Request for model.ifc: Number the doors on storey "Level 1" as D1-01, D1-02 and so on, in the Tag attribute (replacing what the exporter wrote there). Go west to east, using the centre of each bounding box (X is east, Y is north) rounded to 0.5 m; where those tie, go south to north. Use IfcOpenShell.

First a look at what the model holds.

```python
import ifcopenshell
import ifcopenshell.util.element
import ifcopenshell.util.placement

model = ifcopenshell.open("model.ifc")
print(model.schema)
storey = next(s for s in model.by_type("IfcBuildingStorey") if s.Name == "Level 1")
doors = [e for e in ifcopenshell.util.element.get_decomposition(storey) if e.is_a("IfcDoor")]
for e in sorted(doors, key=lambda e: e.id()):
    origin = ifcopenshell.util.placement.get_local_placement(e.ObjectPlacement)[:3, 3]
    print(e.id(), e.Tag, e.Name, origin.round(2) + 0.0, sep=" | ")
```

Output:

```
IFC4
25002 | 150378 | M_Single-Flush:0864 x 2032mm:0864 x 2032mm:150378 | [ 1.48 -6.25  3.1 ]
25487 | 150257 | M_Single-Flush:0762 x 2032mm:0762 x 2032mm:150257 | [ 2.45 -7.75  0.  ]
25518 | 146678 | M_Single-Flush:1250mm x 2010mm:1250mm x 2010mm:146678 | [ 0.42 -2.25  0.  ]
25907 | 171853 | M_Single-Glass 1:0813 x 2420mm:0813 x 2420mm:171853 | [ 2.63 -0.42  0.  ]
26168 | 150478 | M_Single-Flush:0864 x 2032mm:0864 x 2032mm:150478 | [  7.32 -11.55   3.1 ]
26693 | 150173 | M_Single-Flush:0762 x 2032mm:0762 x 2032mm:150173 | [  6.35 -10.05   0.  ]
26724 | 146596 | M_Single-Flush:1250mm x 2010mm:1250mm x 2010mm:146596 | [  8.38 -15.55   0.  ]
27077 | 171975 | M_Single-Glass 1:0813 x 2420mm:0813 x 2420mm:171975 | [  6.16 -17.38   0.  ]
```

```python
import ifcopenshell
import ifcopenshell.geom
import ifcopenshell.util.element
import ifcopenshell.util.shape

model = ifcopenshell.open("model.ifc")
settings = ifcopenshell.geom.settings()
settings.set("use-world-coords", True)


def centre(element):
    shape = ifcopenshell.geom.create_shape(settings, element)
    return ifcopenshell.util.shape.get_bbox_centroid(shape.geometry)


storey = next(s for s in model.by_type("IfcBuildingStorey") if s.Name == "Level 1")
doors = [e for e in ifcopenshell.util.element.get_decomposition(storey) if e.is_a("IfcDoor")]

# Insertion points can sit at a corner or the storey origin, so sort by the geometry (in metres).
centres = {e: centre(e) for e in doors}
doors.sort(key=lambda e: (round(centres[e][0] / 0.5), centres[e][1]))

for i, e in enumerate(doors, start=1):
    number = f"D1-{i:02d}"
    e.Tag = number
    print(e.id(), number)

model.write("model_edited.ifc")
```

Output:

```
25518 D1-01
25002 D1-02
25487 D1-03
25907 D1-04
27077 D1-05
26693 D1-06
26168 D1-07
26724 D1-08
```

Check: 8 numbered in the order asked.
